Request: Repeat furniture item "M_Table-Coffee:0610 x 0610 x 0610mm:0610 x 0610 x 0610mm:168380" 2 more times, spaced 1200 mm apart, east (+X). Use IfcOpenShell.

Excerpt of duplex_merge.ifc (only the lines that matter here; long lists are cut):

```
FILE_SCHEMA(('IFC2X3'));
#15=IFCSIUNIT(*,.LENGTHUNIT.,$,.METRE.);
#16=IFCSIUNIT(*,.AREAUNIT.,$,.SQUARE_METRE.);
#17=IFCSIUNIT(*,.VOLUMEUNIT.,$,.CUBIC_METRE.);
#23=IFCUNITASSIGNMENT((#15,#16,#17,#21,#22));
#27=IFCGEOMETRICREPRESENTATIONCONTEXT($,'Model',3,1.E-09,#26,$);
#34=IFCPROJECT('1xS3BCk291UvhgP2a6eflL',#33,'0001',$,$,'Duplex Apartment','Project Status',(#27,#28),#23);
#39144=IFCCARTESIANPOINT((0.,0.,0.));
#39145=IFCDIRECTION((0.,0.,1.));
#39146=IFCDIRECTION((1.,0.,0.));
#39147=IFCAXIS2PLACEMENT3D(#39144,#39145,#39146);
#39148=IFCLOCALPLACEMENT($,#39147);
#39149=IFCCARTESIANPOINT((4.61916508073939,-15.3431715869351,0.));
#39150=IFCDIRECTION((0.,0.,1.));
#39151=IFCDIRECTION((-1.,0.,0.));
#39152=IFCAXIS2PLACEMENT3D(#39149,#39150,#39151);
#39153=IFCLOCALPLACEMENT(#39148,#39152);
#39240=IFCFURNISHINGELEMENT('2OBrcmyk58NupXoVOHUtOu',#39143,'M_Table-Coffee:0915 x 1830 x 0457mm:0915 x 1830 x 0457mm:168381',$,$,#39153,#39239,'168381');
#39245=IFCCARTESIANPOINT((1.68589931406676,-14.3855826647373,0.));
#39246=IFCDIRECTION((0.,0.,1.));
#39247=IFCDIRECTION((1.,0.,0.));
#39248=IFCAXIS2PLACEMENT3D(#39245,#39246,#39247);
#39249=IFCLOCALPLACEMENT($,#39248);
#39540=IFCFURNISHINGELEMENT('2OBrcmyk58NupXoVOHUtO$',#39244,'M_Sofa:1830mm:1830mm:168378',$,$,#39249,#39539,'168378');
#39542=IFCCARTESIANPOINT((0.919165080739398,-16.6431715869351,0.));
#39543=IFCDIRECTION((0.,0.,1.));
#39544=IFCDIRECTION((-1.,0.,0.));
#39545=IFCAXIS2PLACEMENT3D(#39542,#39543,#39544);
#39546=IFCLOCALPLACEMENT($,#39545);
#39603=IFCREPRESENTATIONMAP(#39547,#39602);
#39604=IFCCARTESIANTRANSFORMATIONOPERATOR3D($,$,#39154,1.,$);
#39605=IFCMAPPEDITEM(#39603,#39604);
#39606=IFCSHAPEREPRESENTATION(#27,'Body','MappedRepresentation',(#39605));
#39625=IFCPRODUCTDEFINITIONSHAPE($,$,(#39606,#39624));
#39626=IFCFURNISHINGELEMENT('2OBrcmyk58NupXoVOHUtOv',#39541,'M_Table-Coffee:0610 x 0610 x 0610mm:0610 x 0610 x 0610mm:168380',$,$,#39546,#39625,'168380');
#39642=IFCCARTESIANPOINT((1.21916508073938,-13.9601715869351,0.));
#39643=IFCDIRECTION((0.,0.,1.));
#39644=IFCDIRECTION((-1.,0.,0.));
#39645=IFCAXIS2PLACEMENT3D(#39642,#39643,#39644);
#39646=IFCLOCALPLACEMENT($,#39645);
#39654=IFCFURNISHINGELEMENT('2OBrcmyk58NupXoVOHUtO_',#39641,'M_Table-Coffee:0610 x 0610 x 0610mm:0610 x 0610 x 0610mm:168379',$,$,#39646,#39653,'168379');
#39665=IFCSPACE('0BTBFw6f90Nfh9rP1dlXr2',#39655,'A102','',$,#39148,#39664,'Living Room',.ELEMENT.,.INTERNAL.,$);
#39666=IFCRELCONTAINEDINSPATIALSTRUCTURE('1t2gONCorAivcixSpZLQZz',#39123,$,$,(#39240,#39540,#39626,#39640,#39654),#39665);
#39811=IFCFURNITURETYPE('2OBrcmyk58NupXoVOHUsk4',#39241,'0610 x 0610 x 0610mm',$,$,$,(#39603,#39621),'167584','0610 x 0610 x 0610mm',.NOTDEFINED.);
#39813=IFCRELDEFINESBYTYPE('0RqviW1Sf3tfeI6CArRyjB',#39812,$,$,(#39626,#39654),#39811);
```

```python
import numpy as np
import ifcopenshell
import ifcopenshell.api.geometry
import ifcopenshell.api.root
import ifcopenshell.util.element
import ifcopenshell.util.placement
import ifcopenshell.util.unit

model = ifcopenshell.open("duplex_merge.ifc")
unit_scale = ifcopenshell.util.unit.calculate_unit_scale(model)


def reuse_history(source, copy):
    """copy_class also copies each property set's owner history, people and application; keep the originals."""
    for rel in copy.IsDefinedBy:
        if rel.is_a("IfcRelDefinesByProperties") and (history := rel.RelatingPropertyDefinition.OwnerHistory):
            rel.RelatingPropertyDefinition.OwnerHistory = source.OwnerHistory
            ifcopenshell.util.element.remove_deep2(model, history)


source = model.by_id(39626)
base = ifcopenshell.util.placement.get_local_placement(source.ObjectPlacement)
step = np.array([1.0, 0.0, 0.0]) * 1.2 / unit_scale

for i in range(1, 3):
    copy = ifcopenshell.api.root.copy_class(model, product=source)
    copy.Representation = ifcopenshell.util.element.copy_deep(
        model, source.Representation, exclude=["IfcGeometricRepresentationContext", "IfcRepresentationMap"]
    )
    copy.Name = "M_Table-Coffee:0610 x 0610 x 0610mm:0610 x 0610 x 0610mm"
    copy.Tag = None
    reuse_history(source, copy)
    matrix = base.copy()
    matrix[:3, 3] += i * step
    print("added at", matrix[:3, 3].round(3) + 0.0)
    ifcopenshell.api.geometry.edit_object_placement(model, product=copy, matrix=matrix, is_si=False)

model.write("duplex_merge-out.ifc")
```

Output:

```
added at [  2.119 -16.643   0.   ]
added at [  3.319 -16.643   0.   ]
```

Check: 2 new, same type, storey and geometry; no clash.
